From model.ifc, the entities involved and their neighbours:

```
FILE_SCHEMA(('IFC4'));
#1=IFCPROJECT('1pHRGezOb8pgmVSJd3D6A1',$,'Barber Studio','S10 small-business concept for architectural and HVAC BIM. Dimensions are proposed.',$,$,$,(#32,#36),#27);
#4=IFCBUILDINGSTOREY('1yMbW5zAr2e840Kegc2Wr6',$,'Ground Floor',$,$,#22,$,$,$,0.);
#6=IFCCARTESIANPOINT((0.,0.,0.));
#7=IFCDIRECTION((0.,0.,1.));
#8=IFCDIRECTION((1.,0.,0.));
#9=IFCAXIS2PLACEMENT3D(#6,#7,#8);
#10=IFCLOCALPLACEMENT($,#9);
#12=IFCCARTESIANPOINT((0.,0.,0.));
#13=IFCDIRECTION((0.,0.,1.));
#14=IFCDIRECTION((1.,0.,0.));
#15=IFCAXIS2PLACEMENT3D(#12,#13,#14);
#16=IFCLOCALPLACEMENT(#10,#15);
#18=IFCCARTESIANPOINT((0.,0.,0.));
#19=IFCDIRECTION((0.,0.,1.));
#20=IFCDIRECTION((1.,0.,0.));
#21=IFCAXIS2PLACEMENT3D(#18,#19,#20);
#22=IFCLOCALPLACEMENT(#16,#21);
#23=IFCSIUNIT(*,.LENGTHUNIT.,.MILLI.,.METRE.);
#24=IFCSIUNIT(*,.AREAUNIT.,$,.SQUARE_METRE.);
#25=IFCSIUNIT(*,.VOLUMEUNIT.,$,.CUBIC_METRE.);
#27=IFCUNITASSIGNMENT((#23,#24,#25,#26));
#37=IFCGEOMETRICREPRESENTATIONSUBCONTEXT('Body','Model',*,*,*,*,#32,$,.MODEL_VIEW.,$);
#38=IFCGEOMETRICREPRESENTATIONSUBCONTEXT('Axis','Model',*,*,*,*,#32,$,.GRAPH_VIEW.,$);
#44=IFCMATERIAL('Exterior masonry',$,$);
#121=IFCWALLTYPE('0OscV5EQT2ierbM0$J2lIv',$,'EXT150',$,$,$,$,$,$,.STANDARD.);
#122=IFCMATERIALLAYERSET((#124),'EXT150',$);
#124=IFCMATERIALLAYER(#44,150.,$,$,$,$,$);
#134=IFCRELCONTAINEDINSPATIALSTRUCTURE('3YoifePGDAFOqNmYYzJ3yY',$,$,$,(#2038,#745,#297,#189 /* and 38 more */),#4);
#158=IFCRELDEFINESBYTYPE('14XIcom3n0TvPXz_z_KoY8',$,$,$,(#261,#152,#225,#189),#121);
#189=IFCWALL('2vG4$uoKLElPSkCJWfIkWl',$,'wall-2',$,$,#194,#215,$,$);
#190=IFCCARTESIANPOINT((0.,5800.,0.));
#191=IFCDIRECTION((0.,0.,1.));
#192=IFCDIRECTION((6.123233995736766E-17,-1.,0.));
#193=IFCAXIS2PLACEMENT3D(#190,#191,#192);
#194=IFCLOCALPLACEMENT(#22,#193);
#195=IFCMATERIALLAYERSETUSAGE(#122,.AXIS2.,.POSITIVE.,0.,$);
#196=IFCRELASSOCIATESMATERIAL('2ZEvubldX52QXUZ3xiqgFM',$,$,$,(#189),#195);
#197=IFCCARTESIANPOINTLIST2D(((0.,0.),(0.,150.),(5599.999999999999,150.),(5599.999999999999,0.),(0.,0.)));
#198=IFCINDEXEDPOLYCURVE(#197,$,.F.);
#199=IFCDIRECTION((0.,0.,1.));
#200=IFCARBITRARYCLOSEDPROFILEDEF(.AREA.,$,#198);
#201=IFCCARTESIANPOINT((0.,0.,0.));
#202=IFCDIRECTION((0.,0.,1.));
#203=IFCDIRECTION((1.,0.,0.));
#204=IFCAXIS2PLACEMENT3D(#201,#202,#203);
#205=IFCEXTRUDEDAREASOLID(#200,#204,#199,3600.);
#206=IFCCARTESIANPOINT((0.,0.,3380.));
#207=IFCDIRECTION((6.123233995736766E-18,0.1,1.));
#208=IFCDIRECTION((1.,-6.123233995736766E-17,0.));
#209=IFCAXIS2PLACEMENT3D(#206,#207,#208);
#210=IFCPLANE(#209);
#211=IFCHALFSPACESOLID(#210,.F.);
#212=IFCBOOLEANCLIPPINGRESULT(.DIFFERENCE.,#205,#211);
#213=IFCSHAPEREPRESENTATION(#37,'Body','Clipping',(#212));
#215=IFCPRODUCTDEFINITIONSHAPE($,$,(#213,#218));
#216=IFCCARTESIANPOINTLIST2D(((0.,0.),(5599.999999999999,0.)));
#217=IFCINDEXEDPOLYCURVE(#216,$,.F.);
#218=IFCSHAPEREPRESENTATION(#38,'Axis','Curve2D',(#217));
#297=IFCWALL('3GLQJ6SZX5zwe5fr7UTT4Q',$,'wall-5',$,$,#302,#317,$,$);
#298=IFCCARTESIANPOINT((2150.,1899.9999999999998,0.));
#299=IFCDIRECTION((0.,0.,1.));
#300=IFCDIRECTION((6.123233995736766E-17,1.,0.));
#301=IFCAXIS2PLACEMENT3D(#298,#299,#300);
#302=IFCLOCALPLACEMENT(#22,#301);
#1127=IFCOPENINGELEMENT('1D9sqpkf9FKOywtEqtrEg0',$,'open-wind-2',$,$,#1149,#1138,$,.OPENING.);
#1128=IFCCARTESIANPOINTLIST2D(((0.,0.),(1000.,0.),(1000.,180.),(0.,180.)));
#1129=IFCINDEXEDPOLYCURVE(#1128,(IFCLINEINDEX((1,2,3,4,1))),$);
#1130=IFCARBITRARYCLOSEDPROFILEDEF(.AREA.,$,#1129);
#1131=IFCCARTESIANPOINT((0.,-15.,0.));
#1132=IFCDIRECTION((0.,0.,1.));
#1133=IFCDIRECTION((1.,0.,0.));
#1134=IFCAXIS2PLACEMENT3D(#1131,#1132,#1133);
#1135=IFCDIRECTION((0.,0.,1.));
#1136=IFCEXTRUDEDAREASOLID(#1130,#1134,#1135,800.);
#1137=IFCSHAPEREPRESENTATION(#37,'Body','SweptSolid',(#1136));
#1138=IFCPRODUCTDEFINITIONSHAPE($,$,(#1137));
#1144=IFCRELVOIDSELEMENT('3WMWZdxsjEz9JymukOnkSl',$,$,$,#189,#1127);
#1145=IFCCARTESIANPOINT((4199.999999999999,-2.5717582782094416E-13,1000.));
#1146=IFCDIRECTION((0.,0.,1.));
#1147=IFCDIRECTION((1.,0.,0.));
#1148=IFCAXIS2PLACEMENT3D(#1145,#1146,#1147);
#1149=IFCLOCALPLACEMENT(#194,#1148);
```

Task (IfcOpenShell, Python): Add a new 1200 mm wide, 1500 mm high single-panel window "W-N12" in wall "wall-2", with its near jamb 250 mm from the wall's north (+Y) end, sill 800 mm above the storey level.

```python
import numpy as np
import ifcopenshell
import ifcopenshell.api.feature
import ifcopenshell.api.geometry
import ifcopenshell.api.root
import ifcopenshell.api.spatial
import ifcopenshell.geom
import ifcopenshell.util.element
import ifcopenshell.util.placement
import ifcopenshell.util.representation
import ifcopenshell.util.shape
import ifcopenshell.util.unit

model = ifcopenshell.open("model.ifc")
unit_scale = ifcopenshell.util.unit.calculate_unit_scale(model)
settings = ifcopenshell.geom.settings()


def volume(element):
    """Net volume in cubic metres, openings subtracted."""
    shape = ifcopenshell.geom.create_shape(settings, element)
    return ifcopenshell.util.shape.get_volume(shape.geometry)


wall = model.by_id(189)
storey = ifcopenshell.util.element.get_container(wall, ifc_class="IfcBuildingStorey")
context = ifcopenshell.util.representation.get_context(model, "Model", "Body", "MODEL_VIEW")
before = volume(wall)

width, height, from_end, sill = 1.2, 1.5, 0.25, 0.8  # metres

# The wall runs along its own X axis, and the end named is its -X end.
wall_shape = ifcopenshell.geom.create_shape(settings, wall)
x, y, z = ifcopenshell.util.shape.get_vertices(wall_shape.geometry).T
start = x.min() + from_end
face, thickness = float(y.min()), float(y.max() - y.min())
wall_matrix = ifcopenshell.util.placement.get_local_placement(wall.ObjectPlacement)
level = ifcopenshell.util.placement.get_local_placement(storey.ObjectPlacement)[2, 3]


def in_wall(x, y):
    """Placement at x, y metres in the wall's axes, at sill height."""
    matrix = wall_matrix.copy()
    matrix[:, 3] = wall_matrix @ np.array([x / unit_scale, y / unit_scale, 0.0, 1.0])
    matrix[2, 3] = level + sill / unit_scale
    return matrix


# Opening: a box that overshoots both wall faces by 50 mm.
opening = ifcopenshell.api.root.create_entity(model, ifc_class="IfcOpeningElement", predefined_type="OPENING")
box = ifcopenshell.api.geometry.add_wall_representation(
    model, context=context, length=width, height=height, thickness=thickness + 0.1
)
ifcopenshell.api.geometry.assign_representation(model, product=opening, representation=box)
ifcopenshell.api.geometry.edit_object_placement(model, product=opening, matrix=in_wall(start, face - 0.05), is_si=False)
ifcopenshell.api.feature.add_feature(model, feature=opening, element=wall)

window = ifcopenshell.api.root.create_entity(model, ifc_class="IfcWindow", name="W-N12", predefined_type="WINDOW")
window.OverallWidth, window.OverallHeight = width / unit_scale, height / unit_scale
window.PartitioningType = "SINGLE_PANEL"
body = ifcopenshell.api.geometry.add_window_representation(
    model,
    context=context,
    overall_width=window.OverallWidth,
    overall_height=window.OverallHeight,
    partition_type="SINGLE_PANEL",
)
ifcopenshell.api.geometry.assign_representation(model, product=window, representation=body)
ifcopenshell.api.spatial.assign_container(model, products=[window], relating_structure=storey)
ifcopenshell.api.feature.add_filling(model, opening=opening, element=window)

# Centre the window in the wall's thickness.
ifcopenshell.api.geometry.edit_object_placement(model, product=window, matrix=in_wall(start, face), is_si=False)
window_shape = ifcopenshell.geom.create_shape(settings, window)
depth = ifcopenshell.util.shape.get_vertices(window_shape.geometry)[:, 1]
offset = face + thickness / 2 - (depth.min() + depth.max()) / 2
ifcopenshell.api.geometry.edit_object_placement(model, product=window, matrix=in_wall(start, offset), is_si=False)

after = volume(wall)

print(f"wall volume {before:.3f} -> {after:.3f} m3")

model.write("model_edited.ifc")
```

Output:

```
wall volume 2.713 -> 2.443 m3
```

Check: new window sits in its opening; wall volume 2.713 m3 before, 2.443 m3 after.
